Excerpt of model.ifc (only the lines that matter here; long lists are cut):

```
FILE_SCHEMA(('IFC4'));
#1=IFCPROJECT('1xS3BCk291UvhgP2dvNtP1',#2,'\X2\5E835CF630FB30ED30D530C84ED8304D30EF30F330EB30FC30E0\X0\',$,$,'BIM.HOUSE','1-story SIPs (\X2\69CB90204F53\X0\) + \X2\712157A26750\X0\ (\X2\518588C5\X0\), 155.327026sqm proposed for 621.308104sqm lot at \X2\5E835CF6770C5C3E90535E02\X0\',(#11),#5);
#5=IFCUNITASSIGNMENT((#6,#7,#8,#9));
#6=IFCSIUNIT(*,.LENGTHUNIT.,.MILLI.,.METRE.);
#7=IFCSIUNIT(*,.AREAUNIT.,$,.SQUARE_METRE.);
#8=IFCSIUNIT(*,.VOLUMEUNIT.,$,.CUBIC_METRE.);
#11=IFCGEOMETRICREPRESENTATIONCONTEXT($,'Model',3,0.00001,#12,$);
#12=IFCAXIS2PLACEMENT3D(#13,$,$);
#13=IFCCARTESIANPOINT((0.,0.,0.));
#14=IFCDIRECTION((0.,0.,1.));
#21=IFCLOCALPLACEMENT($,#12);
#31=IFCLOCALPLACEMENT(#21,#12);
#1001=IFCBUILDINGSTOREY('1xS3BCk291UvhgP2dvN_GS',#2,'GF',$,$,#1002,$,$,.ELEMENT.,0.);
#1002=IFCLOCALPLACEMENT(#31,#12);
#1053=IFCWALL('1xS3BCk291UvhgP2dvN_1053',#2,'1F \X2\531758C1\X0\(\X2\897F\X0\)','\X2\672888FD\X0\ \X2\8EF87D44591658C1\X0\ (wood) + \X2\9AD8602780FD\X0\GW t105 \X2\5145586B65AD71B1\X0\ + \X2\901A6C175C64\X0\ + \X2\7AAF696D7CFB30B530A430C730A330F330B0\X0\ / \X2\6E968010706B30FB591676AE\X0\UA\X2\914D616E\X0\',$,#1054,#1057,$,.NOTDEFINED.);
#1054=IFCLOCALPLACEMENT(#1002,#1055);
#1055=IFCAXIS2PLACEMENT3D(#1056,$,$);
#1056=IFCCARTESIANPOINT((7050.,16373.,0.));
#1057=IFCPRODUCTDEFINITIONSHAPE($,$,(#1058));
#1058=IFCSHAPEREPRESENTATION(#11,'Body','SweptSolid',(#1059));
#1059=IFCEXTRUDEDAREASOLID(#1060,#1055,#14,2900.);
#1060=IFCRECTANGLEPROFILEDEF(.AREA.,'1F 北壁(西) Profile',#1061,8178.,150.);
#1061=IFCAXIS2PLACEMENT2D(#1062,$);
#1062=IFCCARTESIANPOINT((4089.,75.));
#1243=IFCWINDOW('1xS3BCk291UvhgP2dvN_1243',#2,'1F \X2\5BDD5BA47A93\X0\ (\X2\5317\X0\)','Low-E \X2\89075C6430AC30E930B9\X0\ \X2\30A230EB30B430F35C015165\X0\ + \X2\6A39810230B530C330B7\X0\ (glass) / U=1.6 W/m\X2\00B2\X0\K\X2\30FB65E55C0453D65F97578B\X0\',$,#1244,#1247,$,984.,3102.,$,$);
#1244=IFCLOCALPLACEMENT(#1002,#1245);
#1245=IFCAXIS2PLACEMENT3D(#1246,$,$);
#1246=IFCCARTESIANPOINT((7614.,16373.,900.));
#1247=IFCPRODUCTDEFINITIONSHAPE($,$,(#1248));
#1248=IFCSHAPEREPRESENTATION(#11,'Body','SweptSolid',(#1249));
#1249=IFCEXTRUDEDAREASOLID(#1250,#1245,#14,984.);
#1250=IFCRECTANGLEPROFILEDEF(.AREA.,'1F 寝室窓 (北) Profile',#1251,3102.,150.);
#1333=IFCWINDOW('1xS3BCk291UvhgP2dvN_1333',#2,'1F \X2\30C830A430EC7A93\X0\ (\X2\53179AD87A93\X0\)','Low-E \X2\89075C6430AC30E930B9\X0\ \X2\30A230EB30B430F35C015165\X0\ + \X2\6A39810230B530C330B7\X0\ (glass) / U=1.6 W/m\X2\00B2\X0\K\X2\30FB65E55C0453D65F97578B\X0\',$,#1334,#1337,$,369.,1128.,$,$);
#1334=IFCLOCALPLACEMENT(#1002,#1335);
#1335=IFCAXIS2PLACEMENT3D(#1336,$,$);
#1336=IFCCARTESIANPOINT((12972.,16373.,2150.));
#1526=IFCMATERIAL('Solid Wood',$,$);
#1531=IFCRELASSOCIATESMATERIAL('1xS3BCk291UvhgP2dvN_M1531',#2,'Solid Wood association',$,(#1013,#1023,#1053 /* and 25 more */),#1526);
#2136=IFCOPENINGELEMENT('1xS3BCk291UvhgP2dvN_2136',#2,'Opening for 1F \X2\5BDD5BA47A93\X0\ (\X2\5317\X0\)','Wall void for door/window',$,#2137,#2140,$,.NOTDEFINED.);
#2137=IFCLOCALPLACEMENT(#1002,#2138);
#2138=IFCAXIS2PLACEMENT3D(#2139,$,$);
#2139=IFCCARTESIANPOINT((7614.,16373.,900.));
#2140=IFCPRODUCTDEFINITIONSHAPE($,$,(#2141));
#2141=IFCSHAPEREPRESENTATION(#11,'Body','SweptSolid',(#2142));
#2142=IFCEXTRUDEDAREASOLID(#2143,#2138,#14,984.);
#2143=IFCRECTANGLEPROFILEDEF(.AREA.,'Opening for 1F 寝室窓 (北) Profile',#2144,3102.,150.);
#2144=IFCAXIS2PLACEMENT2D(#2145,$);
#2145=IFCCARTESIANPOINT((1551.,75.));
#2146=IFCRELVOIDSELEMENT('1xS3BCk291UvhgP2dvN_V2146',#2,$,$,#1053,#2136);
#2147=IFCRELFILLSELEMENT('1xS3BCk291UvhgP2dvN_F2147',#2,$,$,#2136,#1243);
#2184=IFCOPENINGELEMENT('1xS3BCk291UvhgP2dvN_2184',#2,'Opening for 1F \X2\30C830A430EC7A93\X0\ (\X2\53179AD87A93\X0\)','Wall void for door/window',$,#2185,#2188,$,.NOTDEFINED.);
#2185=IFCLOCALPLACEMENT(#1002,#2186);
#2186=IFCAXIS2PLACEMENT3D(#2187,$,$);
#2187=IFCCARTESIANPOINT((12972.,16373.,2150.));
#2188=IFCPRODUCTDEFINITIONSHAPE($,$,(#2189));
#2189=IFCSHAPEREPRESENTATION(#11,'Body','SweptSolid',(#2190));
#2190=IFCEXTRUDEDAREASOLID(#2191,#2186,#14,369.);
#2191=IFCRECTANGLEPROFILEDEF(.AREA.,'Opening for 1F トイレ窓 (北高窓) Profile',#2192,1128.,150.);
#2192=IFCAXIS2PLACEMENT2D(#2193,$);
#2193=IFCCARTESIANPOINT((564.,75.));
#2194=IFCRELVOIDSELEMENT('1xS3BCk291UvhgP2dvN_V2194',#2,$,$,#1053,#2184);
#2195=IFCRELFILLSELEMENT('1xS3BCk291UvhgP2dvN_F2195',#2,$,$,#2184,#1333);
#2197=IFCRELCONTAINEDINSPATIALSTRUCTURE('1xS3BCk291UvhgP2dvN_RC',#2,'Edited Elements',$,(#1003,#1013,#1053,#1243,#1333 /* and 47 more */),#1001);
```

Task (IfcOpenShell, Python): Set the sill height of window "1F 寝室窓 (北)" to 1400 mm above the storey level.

```python
import numpy as np
import ifcopenshell
import ifcopenshell.api.geometry
import ifcopenshell.geom
import ifcopenshell.util.element
import ifcopenshell.util.placement
import ifcopenshell.util.shape
import ifcopenshell.util.unit

model = ifcopenshell.open("model.ifc")
unit_scale = ifcopenshell.util.unit.calculate_unit_scale(model)

window = model.by_guid("1xS3BCk291UvhgP2dvN_1243")
opening = window.FillsVoids[0].RelatingOpeningElement
storey = ifcopenshell.util.element.get_container(window, ifc_class="IfcBuildingStorey")
level = ifcopenshell.util.placement.get_local_placement(storey.ObjectPlacement)[2, 3]

# The opening's origin need not be at the sill, so measure its lowest point.
shape = ifcopenshell.geom.create_shape(ifcopenshell.geom.settings(), opening)
bottom = ifcopenshell.util.shape.get_shape_bottom_elevation(shape, shape.geometry) / unit_scale
dz = level + 1400.0 - bottom

shift = np.array([0.0, 0.0, dz])
# The window is not placed relative to its opening, so move both.
for product in (opening, window):
    matrix = ifcopenshell.util.placement.get_local_placement(product.ObjectPlacement)
    matrix[:3, 3] += shift
    ifcopenshell.api.geometry.edit_object_placement(model, product=product, matrix=matrix, is_si=False)

print(f"moved by {dz * unit_scale:+.3f} m")

model.write("model_edited.ifc")
```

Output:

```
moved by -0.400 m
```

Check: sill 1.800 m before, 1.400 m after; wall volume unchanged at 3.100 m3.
